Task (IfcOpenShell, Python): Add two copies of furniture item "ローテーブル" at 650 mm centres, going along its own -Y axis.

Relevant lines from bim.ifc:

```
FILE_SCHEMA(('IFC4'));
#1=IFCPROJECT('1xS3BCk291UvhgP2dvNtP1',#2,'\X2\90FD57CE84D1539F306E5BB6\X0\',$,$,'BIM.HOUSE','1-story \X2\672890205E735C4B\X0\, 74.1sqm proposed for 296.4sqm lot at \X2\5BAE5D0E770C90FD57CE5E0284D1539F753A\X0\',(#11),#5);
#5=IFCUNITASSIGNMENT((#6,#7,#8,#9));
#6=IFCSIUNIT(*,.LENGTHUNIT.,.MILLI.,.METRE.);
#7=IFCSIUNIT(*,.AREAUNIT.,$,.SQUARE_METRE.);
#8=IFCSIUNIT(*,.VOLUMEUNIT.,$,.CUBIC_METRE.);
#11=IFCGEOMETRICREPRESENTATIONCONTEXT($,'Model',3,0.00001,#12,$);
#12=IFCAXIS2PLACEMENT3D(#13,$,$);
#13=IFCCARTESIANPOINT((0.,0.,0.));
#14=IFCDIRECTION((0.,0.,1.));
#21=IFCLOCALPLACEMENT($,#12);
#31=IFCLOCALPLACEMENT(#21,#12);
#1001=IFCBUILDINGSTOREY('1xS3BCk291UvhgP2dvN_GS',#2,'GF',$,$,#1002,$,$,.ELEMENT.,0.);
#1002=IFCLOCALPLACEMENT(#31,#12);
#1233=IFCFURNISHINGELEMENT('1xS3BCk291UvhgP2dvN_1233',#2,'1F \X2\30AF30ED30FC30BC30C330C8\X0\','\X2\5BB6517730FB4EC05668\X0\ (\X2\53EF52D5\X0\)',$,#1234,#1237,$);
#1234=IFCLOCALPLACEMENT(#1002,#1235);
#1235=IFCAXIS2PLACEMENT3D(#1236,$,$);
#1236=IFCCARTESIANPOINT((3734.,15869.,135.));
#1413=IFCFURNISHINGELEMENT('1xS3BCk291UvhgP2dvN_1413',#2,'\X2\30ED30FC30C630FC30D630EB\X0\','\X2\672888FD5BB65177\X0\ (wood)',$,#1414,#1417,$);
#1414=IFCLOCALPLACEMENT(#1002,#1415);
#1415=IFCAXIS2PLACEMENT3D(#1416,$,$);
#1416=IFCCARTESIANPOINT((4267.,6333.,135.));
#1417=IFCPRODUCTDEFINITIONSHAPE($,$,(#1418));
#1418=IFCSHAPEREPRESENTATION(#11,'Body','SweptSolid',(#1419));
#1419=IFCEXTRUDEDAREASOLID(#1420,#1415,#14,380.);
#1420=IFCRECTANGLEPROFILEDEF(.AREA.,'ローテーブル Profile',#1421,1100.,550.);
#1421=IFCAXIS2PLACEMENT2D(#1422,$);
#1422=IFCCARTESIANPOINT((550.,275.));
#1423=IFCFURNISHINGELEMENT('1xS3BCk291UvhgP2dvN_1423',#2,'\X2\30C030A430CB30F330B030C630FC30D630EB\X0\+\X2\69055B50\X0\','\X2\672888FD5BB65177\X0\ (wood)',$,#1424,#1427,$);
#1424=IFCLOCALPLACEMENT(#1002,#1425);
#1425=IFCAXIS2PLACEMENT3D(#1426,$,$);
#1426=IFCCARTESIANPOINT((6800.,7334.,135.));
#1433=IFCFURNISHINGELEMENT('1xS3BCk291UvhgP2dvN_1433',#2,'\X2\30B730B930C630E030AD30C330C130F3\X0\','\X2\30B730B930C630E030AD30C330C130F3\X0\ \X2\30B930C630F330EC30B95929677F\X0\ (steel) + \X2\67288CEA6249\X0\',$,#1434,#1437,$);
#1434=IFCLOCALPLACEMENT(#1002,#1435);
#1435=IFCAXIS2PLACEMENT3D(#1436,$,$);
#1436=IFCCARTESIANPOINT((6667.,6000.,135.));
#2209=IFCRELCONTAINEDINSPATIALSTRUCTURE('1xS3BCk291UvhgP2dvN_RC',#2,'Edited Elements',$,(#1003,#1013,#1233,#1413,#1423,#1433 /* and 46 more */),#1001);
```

```python
import ifcopenshell
import ifcopenshell.api.geometry
import ifcopenshell.api.root
import ifcopenshell.util.element
import ifcopenshell.util.placement

model = ifcopenshell.open("bim.ifc")


def reuse_history(source, copy):
    """copy_class also copies each property set's owner history, people and application; keep the originals."""
    for rel in copy.IsDefinedBy:
        if rel.is_a("IfcRelDefinesByProperties") and (history := rel.RelatingPropertyDefinition.OwnerHistory):
            rel.RelatingPropertyDefinition.OwnerHistory = source.OwnerHistory
            ifcopenshell.util.element.remove_deep2(model, history)


source = model.by_guid("1xS3BCk291UvhgP2dvN_1413")
base = ifcopenshell.util.placement.get_local_placement(source.ObjectPlacement)
step = -base[:3, 1] * 650.0

for i in range(1, 3):
    copy = ifcopenshell.api.root.copy_class(model, product=source)
    copy.Representation = ifcopenshell.util.element.copy_deep(
        model, source.Representation, exclude=["IfcGeometricRepresentationContext", "IfcRepresentationMap"]
    )
    reuse_history(source, copy)
    matrix = base.copy()
    matrix[:3, 3] += i * step
    print("added at", matrix[:3, 3].round(3) + 0.0)
    ifcopenshell.api.geometry.edit_object_placement(model, product=copy, matrix=matrix, is_si=False)

model.write("bim-out.ifc")
```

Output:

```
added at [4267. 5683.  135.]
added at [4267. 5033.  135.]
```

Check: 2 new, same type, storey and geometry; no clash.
